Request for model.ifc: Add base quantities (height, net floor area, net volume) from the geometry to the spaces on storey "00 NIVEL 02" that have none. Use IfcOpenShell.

First a look at what the model holds.

```python
import ifcopenshell
import ifcopenshell.util.element
import ifcopenshell.util.unit

model = ifcopenshell.open("model.ifc")
print(model.schema)
for unit_type in ("LENGTHUNIT", "AREAUNIT", "VOLUMEUNIT"):
    print(unit_type, ifcopenshell.util.unit.calculate_unit_scale(model, unit_type))
storey = next(s for s in model.by_type("IfcBuildingStorey") if s.Name == "00 NIVEL 02")
spaces = [e for e in ifcopenshell.util.element.get_decomposition(storey) if e.is_a("IfcSpace")]
for e in sorted(spaces, key=lambda e: e.id()):
    print(e.id(), e.is_a(), e.Name, list(ifcopenshell.util.element.get_psets(e, qtos_only=True)), sep=" | ")
```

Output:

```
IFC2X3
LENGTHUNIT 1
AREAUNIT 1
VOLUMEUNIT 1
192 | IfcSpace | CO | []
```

```python
import ifcopenshell
import ifcopenshell.api.pset
import ifcopenshell.geom
import ifcopenshell.util.element
import ifcopenshell.util.shape
import ifcopenshell.util.unit

model = ifcopenshell.open("model.ifc")
unit_scale = ifcopenshell.util.unit.calculate_unit_scale(model)
area_scale = ifcopenshell.util.unit.calculate_unit_scale(model, "AREAUNIT")
volume_scale = ifcopenshell.util.unit.calculate_unit_scale(model, "VOLUMEUNIT")
settings = ifcopenshell.geom.settings()

storey = next(s for s in model.by_type("IfcBuildingStorey") if s.Name == "00 NIVEL 02")
spaces = [e for e in ifcopenshell.util.element.get_decomposition(storey) if e.is_a("IfcSpace")]

for e in sorted(spaces, key=lambda e: e.id()):
    if ifcopenshell.util.element.get_psets(e, qtos_only=True, should_inherit=False):
        continue
    # Geometry comes back in metres, in the element's own axes.
    shape = ifcopenshell.geom.create_shape(settings, e)
    values = {
        "Height": ifcopenshell.util.shape.get_z(shape.geometry) / unit_scale,
        "NetFloorArea": ifcopenshell.util.shape.get_footprint_area(shape.geometry) / area_scale,
        "NetVolume": ifcopenshell.util.shape.get_volume(shape.geometry) / volume_scale,
    }
    qto = ifcopenshell.api.pset.add_qto(model, product=e, name="BaseQuantities")
    ifcopenshell.api.pset.edit_qto(model, qto=qto, properties=values)
    print(e.id(), {k: round(v, 3) for k, v in values.items()})

model.write("model_rev.ifc")
```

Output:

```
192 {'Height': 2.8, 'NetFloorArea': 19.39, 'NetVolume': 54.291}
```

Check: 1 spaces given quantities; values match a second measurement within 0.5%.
